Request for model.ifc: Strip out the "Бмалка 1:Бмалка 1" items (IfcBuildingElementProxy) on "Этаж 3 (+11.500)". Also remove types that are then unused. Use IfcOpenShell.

First a look at what the model holds.

```python
import ifcopenshell
import ifcopenshell.util.element

model = ifcopenshell.open("model.ifc")
print(model.schema)
storey = next(s for s in model.by_type("IfcBuildingStorey") if s.Name == "Этаж 3 (+11.500)")
proxies = [e for e in ifcopenshell.util.element.get_decomposition(storey) if e.is_a("IfcBuildingElementProxy")]
seen = {}
for e in proxies:
    element_type = ifcopenshell.util.element.get_type(e)
    name = element_type.Name if element_type not in (None, e) else None
    seen[name] = seen.get(name, 0) + 1
for name, count in sorted(seen.items(), key=str):
    print(count, "x", name)
```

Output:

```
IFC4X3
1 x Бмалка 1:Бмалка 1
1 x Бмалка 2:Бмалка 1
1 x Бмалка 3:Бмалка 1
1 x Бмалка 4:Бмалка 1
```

```python
import ifcopenshell
import ifcopenshell.api.root
import ifcopenshell.util.element

model = ifcopenshell.open("model.ifc")

storey = next(s for s in model.by_type("IfcBuildingStorey") if s.Name == "Этаж 3 (+11.500)")
proxies = [e for e in ifcopenshell.util.element.get_decomposition(storey) if e.is_a("IfcBuildingElementProxy")]
targets = [e for e in proxies if (t := ifcopenshell.util.element.get_type(e)) not in (None, e) and t.Name == "Бмалка 1:Бмалка 1"]
types = {ifcopenshell.util.element.get_type(e) for e in targets} - {None, *targets}

for e in targets:
    ifcopenshell.api.root.remove_product(model, product=e)
print(len(targets), "removed")

unused = [t for t in types if not ifcopenshell.util.element.get_types(t)]
for t in unused:
    ifcopenshell.api.root.remove_product(model, product=t)
print(len(unused), "unused types removed")

model.write("model_edited.ifc")
```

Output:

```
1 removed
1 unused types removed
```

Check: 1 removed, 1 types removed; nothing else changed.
